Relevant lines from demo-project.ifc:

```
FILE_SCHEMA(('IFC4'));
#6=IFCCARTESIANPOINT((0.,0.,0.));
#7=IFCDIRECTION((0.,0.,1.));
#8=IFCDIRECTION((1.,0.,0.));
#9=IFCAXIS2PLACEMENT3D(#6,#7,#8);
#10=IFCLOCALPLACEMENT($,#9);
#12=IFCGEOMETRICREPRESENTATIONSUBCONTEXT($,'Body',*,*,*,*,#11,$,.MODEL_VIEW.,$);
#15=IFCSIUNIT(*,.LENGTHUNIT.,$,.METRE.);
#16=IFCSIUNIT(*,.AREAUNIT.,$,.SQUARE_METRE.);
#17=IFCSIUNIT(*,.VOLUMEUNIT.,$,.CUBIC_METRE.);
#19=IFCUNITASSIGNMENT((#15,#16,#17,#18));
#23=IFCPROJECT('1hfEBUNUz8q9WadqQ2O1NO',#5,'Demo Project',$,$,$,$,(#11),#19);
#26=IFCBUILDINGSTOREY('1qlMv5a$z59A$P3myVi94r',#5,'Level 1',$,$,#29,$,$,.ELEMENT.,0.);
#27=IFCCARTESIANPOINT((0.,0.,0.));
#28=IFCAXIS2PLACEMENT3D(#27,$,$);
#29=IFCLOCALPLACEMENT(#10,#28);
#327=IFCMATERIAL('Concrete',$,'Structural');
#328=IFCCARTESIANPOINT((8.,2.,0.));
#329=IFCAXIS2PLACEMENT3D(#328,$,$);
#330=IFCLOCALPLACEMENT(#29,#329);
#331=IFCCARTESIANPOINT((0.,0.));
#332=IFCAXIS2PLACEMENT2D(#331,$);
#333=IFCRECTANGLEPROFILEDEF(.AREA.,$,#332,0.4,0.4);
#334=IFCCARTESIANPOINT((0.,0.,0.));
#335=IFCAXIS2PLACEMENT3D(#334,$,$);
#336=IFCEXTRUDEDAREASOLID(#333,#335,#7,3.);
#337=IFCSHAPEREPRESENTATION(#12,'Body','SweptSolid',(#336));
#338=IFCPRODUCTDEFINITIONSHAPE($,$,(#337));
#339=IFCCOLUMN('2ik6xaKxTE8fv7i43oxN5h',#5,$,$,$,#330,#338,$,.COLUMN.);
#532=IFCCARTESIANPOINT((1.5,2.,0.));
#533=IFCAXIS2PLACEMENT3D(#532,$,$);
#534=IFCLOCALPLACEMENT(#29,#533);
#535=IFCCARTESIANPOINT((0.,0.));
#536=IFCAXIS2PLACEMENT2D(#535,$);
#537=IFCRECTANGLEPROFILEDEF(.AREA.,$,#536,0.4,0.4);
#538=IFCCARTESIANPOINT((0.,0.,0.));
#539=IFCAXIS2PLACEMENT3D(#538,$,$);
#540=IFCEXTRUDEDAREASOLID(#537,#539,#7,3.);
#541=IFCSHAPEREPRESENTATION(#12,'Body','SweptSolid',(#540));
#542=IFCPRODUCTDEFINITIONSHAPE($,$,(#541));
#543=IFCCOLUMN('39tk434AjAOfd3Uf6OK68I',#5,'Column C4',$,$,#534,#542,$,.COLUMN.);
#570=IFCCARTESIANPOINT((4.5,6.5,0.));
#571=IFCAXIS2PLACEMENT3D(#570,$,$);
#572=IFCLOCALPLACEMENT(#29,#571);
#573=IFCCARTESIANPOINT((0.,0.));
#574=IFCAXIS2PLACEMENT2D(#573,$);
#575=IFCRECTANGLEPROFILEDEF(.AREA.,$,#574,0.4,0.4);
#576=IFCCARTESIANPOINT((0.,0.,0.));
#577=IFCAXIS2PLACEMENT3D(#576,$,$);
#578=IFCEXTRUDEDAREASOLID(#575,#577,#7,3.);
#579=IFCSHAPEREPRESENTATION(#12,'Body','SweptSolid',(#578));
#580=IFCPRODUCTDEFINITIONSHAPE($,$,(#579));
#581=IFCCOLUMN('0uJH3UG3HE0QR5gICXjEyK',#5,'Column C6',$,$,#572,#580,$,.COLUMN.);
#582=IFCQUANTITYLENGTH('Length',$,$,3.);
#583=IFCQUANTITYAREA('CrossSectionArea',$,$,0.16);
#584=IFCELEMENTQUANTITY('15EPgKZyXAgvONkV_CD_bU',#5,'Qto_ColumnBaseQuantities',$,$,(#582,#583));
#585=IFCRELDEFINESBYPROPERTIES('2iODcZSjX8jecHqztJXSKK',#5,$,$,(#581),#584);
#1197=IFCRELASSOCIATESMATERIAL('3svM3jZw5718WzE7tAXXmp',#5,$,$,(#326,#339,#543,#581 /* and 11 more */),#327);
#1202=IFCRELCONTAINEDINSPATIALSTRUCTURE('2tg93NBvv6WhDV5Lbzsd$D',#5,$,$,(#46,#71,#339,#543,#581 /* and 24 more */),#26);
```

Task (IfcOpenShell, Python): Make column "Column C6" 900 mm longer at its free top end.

```python
import ifcopenshell
import ifcopenshell.api.pset
import ifcopenshell.util.element
import ifcopenshell.util.unit

model = ifcopenshell.open("demo-project.ifc")
unit_scale = ifcopenshell.util.unit.calculate_unit_scale(model)

member = model.by_guid("0uJH3UG3HE0QR5gICXjEyK")
change = 0.9 / unit_scale

# The extrusion runs towards the end named, so only its depth changes.
body = next(r for r in member.Representation.Representations if r.RepresentationIdentifier == "Body")
solid = body.Items[0]
old_length = solid.Depth
solid.Depth += change

# Update the stored length and volume.
qto = model.by_id(ifcopenshell.util.element.get_pset(member, "Qto_ColumnBaseQuantities", should_inherit=False)["id"])
ifcopenshell.api.pset.edit_qto(model, qto=qto, properties={"Length": solid.Depth})

print(f"length {old_length:g} -> {solid.Depth:g}")

model.write("demo-project_updated.ifc")
```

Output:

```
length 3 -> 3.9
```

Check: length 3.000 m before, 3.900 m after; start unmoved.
